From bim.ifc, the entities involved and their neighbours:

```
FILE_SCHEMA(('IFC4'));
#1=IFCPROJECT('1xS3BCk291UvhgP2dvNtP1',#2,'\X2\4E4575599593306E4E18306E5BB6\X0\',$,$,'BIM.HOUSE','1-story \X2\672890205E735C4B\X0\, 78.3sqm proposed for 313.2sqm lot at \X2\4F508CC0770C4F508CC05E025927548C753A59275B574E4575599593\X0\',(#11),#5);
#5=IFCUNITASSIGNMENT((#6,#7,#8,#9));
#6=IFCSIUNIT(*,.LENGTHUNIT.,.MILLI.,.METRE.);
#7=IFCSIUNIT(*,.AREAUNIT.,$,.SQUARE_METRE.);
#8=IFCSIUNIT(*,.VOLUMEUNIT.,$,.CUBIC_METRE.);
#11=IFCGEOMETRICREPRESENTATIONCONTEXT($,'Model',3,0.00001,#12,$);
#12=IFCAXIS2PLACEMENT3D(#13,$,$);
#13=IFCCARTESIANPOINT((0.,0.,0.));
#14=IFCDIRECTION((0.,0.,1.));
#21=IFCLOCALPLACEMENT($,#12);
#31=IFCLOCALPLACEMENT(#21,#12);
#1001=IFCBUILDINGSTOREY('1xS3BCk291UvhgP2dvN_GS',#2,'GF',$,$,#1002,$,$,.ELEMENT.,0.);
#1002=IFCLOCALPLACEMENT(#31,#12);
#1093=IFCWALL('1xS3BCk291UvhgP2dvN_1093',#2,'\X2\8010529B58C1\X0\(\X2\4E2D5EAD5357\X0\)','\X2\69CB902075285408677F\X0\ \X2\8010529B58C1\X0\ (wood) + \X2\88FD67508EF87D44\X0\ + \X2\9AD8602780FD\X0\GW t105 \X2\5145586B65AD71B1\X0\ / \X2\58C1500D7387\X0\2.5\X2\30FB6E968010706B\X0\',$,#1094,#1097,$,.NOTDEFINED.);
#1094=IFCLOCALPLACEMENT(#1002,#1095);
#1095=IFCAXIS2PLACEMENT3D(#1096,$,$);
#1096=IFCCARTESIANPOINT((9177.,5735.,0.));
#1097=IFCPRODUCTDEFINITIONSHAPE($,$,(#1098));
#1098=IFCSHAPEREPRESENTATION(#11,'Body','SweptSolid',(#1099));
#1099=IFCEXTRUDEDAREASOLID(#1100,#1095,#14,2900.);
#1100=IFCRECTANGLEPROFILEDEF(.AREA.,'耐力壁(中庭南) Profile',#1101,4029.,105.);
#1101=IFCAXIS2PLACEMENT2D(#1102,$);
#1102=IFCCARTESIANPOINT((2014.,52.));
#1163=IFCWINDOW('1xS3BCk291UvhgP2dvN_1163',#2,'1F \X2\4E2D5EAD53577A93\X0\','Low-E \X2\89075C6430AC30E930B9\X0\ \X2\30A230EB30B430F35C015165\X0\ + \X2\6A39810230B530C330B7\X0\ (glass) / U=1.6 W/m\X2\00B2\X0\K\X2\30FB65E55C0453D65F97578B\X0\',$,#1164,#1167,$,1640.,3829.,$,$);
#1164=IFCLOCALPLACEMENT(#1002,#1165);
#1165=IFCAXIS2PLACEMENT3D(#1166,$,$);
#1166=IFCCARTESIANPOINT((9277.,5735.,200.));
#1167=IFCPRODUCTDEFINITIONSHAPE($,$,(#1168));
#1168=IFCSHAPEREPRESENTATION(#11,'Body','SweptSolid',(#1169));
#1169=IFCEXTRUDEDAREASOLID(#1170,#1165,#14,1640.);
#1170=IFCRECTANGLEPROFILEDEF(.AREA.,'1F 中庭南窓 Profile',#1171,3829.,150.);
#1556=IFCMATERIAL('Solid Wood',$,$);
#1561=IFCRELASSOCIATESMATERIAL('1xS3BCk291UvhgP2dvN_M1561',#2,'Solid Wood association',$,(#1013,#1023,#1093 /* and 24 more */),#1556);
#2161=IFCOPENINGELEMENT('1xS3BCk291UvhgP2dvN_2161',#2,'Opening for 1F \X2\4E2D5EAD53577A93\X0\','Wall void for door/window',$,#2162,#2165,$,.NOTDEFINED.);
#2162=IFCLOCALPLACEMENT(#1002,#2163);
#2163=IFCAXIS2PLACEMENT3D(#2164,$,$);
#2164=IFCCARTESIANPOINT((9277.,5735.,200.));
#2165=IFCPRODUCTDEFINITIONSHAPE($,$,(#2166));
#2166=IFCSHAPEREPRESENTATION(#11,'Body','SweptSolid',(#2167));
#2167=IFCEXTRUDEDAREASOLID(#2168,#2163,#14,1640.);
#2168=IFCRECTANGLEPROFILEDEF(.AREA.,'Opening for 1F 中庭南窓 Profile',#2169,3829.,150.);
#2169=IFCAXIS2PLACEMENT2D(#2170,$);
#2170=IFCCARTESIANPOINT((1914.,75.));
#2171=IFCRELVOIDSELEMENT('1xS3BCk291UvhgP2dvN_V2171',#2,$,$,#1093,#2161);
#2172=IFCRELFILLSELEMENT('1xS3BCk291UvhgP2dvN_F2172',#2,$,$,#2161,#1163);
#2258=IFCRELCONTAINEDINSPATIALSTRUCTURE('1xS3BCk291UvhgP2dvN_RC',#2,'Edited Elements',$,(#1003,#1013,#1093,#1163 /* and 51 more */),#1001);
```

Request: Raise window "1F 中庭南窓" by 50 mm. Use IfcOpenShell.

```python
import numpy as np
import ifcopenshell
import ifcopenshell.api.geometry
import ifcopenshell.util.placement
import ifcopenshell.util.unit

model = ifcopenshell.open("bim.ifc")
unit_scale = ifcopenshell.util.unit.calculate_unit_scale(model)

window = model.by_guid("1xS3BCk291UvhgP2dvN_1163")
opening = window.FillsVoids[0].RelatingOpeningElement
dz = 0.05 / unit_scale

shift = np.array([0.0, 0.0, dz])
# The window is not placed relative to its opening, so move both.
for product in (opening, window):
    matrix = ifcopenshell.util.placement.get_local_placement(product.ObjectPlacement)
    matrix[:3, 3] += shift
    ifcopenshell.api.geometry.edit_object_placement(model, product=product, matrix=matrix, is_si=False)

print(f"moved by {dz * unit_scale:+.3f} m")

model.write("bim_rev.ifc")
```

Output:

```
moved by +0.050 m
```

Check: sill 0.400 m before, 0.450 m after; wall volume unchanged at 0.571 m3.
